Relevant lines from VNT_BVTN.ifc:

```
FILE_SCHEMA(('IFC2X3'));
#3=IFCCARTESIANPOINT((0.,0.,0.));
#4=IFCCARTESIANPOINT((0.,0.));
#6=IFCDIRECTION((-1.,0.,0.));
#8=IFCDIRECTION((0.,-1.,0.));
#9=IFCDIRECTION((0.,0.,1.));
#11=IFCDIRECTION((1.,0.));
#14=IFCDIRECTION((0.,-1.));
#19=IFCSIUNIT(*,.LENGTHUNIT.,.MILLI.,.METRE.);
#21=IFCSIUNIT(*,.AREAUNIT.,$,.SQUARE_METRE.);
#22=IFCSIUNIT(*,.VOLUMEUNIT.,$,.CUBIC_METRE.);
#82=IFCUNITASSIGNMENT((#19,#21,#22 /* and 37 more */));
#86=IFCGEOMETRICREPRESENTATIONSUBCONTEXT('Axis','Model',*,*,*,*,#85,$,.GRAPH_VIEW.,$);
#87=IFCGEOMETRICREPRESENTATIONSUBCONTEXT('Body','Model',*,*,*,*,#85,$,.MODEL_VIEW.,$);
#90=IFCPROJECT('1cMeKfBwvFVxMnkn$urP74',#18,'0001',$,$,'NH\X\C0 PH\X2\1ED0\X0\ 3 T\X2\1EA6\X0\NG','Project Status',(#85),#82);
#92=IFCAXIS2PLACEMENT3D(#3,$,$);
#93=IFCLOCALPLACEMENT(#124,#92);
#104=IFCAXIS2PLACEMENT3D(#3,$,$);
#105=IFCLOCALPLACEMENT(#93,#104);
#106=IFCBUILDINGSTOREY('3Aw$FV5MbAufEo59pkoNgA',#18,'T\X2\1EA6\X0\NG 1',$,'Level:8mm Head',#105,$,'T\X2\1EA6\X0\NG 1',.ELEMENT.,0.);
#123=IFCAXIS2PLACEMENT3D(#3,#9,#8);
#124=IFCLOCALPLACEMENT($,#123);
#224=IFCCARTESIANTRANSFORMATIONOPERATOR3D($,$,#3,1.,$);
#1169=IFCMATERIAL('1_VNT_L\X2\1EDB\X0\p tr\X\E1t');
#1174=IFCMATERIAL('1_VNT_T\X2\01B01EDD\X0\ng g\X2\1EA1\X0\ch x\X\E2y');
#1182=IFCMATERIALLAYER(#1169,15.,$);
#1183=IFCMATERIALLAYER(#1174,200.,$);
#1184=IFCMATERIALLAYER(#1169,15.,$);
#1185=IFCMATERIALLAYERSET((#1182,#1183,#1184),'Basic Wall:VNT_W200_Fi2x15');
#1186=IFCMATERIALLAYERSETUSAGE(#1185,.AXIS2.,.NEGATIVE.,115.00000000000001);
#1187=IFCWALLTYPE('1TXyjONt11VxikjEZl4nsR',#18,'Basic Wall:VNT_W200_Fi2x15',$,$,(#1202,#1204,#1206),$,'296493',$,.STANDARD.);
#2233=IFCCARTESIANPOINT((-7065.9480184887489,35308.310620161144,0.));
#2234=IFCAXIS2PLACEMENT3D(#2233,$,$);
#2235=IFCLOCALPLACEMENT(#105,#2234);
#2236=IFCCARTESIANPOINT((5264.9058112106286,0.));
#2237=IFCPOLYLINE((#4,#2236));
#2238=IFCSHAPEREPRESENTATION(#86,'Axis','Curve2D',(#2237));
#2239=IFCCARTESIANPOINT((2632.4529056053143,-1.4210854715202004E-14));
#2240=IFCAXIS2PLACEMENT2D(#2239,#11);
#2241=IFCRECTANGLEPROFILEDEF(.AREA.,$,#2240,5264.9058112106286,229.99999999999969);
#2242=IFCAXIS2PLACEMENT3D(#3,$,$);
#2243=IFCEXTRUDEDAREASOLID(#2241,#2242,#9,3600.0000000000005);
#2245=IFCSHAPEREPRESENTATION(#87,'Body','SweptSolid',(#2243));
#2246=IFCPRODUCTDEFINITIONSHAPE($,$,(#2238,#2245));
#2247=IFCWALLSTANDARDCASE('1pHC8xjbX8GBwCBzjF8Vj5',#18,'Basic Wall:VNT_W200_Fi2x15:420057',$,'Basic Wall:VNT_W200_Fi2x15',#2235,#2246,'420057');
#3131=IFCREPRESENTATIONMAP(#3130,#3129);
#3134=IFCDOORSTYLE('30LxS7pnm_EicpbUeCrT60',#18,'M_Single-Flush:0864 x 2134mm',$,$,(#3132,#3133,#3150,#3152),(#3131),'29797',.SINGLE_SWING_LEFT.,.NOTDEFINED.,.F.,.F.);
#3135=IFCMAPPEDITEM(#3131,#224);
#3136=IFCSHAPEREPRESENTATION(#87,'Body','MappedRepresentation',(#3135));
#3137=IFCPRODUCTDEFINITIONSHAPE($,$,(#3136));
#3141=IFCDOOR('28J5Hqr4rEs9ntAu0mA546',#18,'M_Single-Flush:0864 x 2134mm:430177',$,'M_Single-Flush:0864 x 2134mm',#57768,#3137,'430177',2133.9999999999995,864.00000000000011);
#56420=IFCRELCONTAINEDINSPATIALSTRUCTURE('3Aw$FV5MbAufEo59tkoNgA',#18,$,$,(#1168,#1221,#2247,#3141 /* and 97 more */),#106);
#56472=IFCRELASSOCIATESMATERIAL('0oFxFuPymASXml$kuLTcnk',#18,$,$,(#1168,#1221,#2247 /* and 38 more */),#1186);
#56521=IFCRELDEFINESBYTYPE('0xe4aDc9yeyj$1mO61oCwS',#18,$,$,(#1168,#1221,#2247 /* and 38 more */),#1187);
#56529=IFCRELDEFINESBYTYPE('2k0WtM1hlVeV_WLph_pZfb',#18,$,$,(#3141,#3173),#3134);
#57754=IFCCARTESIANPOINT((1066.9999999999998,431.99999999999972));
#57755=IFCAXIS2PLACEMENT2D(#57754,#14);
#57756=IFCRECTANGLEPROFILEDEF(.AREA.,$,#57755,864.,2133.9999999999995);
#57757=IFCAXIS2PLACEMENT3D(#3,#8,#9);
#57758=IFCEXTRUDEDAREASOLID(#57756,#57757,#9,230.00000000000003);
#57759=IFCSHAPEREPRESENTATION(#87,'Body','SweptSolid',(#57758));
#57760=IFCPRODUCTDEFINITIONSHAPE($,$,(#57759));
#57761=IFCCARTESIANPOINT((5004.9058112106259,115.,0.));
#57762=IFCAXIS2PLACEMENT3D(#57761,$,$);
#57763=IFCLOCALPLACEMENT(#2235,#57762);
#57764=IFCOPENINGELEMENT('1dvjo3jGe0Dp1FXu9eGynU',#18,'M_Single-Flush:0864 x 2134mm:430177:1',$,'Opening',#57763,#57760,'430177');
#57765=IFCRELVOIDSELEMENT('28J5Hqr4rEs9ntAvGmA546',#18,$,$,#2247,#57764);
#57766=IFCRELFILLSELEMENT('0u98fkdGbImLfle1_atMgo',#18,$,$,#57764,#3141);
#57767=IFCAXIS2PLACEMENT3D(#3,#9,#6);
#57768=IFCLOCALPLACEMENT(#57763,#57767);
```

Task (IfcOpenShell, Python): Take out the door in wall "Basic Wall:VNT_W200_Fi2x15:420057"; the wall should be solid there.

```python
import ifcopenshell
import ifcopenshell.api.feature
import ifcopenshell.api.root
import ifcopenshell.geom
import ifcopenshell.util.shape

model = ifcopenshell.open("VNT_BVTN.ifc")
settings = ifcopenshell.geom.settings()


def volume(element):
    """Net volume in cubic metres, openings subtracted."""
    shape = ifcopenshell.geom.create_shape(settings, element)
    return ifcopenshell.util.shape.get_volume(shape.geometry)


door = model.by_guid("28J5Hqr4rEs9ntAu0mA546")
opening = door.FillsVoids[0].RelatingOpeningElement
wall = opening.VoidsElements[0].RelatingBuildingElement
before = volume(wall)

ifcopenshell.api.root.remove_product(model, product=door)
ifcopenshell.api.feature.remove_feature(model, feature=opening)

after = volume(wall)

print(f"wall volume {before:.3f} -> {after:.3f} m3")

model.write("VNT_BVTN_edited.ifc")
```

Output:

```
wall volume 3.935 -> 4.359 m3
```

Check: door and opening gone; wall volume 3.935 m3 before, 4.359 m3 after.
